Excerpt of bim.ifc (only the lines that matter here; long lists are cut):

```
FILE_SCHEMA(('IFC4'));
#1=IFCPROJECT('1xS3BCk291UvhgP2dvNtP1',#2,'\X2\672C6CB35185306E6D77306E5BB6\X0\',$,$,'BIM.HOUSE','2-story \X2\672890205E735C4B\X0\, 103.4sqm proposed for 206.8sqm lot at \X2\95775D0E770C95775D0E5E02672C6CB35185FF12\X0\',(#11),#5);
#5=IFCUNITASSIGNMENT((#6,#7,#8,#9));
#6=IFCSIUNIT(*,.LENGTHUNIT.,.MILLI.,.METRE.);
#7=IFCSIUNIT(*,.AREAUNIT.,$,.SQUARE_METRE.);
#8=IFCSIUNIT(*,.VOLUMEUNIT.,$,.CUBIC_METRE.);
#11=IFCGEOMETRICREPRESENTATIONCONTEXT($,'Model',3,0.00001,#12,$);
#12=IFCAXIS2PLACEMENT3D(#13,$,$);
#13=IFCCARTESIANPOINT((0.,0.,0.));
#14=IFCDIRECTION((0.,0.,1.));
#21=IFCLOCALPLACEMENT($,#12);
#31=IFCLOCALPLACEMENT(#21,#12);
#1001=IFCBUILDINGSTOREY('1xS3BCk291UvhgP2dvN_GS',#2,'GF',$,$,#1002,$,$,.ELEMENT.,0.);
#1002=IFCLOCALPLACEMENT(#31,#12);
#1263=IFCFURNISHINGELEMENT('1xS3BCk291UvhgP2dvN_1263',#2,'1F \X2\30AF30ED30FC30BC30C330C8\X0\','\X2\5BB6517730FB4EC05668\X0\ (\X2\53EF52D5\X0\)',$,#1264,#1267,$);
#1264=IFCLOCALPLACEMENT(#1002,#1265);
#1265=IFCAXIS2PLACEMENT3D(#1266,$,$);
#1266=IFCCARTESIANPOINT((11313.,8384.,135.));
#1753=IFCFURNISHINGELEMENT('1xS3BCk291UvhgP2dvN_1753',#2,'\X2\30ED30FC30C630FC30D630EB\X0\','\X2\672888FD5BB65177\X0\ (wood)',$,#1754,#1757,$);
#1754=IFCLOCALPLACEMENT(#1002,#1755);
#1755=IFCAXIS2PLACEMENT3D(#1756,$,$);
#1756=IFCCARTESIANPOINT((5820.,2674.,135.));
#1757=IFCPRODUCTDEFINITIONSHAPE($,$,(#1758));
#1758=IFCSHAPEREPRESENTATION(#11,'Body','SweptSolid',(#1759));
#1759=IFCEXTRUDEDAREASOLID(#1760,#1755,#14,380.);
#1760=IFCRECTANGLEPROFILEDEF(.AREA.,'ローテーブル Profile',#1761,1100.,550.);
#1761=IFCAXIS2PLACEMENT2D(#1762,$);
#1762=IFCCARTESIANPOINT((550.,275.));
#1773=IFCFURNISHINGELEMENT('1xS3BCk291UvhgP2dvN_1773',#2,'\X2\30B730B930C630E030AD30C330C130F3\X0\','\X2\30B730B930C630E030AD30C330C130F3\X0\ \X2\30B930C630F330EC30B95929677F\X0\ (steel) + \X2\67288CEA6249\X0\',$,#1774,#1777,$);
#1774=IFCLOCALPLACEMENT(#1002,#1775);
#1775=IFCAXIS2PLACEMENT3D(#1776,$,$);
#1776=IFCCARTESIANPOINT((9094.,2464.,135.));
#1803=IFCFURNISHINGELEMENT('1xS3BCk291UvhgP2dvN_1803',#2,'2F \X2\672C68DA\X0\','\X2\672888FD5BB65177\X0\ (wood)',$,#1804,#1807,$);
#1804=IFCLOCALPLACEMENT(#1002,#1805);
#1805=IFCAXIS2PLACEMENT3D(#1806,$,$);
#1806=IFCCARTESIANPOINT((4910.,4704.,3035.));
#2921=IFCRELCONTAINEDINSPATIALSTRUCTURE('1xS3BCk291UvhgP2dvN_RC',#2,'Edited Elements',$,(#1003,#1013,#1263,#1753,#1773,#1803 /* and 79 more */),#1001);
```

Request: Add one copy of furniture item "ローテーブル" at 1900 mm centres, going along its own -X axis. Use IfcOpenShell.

```python
import ifcopenshell
import ifcopenshell.api.geometry
import ifcopenshell.api.root
import ifcopenshell.util.element
import ifcopenshell.util.placement
import ifcopenshell.util.unit

model = ifcopenshell.open("bim.ifc")
unit_scale = ifcopenshell.util.unit.calculate_unit_scale(model)


def reuse_history(source, copy):
    """copy_class also copies each property set's owner history, people and application; keep the originals."""
    for rel in copy.IsDefinedBy:
        if rel.is_a("IfcRelDefinesByProperties") and (history := rel.RelatingPropertyDefinition.OwnerHistory):
            rel.RelatingPropertyDefinition.OwnerHistory = source.OwnerHistory
            ifcopenshell.util.element.remove_deep2(model, history)


source = model.by_guid("1xS3BCk291UvhgP2dvN_1753")
base = ifcopenshell.util.placement.get_local_placement(source.ObjectPlacement)
step = -base[:3, 0] * 1.9 / unit_scale

for i in range(1, 2):
    copy = ifcopenshell.api.root.copy_class(model, product=source)
    copy.Representation = ifcopenshell.util.element.copy_deep(
        model, source.Representation, exclude=["IfcGeometricRepresentationContext", "IfcRepresentationMap"]
    )
    reuse_history(source, copy)
    matrix = base.copy()
    matrix[:3, 3] += i * step
    print("added at", matrix[:3, 3].round(3) + 0.0)
    ifcopenshell.api.geometry.edit_object_placement(model, product=copy, matrix=matrix, is_si=False)

model.write("bim_v2.ifc")
```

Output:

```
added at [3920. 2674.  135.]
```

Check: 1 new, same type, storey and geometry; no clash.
